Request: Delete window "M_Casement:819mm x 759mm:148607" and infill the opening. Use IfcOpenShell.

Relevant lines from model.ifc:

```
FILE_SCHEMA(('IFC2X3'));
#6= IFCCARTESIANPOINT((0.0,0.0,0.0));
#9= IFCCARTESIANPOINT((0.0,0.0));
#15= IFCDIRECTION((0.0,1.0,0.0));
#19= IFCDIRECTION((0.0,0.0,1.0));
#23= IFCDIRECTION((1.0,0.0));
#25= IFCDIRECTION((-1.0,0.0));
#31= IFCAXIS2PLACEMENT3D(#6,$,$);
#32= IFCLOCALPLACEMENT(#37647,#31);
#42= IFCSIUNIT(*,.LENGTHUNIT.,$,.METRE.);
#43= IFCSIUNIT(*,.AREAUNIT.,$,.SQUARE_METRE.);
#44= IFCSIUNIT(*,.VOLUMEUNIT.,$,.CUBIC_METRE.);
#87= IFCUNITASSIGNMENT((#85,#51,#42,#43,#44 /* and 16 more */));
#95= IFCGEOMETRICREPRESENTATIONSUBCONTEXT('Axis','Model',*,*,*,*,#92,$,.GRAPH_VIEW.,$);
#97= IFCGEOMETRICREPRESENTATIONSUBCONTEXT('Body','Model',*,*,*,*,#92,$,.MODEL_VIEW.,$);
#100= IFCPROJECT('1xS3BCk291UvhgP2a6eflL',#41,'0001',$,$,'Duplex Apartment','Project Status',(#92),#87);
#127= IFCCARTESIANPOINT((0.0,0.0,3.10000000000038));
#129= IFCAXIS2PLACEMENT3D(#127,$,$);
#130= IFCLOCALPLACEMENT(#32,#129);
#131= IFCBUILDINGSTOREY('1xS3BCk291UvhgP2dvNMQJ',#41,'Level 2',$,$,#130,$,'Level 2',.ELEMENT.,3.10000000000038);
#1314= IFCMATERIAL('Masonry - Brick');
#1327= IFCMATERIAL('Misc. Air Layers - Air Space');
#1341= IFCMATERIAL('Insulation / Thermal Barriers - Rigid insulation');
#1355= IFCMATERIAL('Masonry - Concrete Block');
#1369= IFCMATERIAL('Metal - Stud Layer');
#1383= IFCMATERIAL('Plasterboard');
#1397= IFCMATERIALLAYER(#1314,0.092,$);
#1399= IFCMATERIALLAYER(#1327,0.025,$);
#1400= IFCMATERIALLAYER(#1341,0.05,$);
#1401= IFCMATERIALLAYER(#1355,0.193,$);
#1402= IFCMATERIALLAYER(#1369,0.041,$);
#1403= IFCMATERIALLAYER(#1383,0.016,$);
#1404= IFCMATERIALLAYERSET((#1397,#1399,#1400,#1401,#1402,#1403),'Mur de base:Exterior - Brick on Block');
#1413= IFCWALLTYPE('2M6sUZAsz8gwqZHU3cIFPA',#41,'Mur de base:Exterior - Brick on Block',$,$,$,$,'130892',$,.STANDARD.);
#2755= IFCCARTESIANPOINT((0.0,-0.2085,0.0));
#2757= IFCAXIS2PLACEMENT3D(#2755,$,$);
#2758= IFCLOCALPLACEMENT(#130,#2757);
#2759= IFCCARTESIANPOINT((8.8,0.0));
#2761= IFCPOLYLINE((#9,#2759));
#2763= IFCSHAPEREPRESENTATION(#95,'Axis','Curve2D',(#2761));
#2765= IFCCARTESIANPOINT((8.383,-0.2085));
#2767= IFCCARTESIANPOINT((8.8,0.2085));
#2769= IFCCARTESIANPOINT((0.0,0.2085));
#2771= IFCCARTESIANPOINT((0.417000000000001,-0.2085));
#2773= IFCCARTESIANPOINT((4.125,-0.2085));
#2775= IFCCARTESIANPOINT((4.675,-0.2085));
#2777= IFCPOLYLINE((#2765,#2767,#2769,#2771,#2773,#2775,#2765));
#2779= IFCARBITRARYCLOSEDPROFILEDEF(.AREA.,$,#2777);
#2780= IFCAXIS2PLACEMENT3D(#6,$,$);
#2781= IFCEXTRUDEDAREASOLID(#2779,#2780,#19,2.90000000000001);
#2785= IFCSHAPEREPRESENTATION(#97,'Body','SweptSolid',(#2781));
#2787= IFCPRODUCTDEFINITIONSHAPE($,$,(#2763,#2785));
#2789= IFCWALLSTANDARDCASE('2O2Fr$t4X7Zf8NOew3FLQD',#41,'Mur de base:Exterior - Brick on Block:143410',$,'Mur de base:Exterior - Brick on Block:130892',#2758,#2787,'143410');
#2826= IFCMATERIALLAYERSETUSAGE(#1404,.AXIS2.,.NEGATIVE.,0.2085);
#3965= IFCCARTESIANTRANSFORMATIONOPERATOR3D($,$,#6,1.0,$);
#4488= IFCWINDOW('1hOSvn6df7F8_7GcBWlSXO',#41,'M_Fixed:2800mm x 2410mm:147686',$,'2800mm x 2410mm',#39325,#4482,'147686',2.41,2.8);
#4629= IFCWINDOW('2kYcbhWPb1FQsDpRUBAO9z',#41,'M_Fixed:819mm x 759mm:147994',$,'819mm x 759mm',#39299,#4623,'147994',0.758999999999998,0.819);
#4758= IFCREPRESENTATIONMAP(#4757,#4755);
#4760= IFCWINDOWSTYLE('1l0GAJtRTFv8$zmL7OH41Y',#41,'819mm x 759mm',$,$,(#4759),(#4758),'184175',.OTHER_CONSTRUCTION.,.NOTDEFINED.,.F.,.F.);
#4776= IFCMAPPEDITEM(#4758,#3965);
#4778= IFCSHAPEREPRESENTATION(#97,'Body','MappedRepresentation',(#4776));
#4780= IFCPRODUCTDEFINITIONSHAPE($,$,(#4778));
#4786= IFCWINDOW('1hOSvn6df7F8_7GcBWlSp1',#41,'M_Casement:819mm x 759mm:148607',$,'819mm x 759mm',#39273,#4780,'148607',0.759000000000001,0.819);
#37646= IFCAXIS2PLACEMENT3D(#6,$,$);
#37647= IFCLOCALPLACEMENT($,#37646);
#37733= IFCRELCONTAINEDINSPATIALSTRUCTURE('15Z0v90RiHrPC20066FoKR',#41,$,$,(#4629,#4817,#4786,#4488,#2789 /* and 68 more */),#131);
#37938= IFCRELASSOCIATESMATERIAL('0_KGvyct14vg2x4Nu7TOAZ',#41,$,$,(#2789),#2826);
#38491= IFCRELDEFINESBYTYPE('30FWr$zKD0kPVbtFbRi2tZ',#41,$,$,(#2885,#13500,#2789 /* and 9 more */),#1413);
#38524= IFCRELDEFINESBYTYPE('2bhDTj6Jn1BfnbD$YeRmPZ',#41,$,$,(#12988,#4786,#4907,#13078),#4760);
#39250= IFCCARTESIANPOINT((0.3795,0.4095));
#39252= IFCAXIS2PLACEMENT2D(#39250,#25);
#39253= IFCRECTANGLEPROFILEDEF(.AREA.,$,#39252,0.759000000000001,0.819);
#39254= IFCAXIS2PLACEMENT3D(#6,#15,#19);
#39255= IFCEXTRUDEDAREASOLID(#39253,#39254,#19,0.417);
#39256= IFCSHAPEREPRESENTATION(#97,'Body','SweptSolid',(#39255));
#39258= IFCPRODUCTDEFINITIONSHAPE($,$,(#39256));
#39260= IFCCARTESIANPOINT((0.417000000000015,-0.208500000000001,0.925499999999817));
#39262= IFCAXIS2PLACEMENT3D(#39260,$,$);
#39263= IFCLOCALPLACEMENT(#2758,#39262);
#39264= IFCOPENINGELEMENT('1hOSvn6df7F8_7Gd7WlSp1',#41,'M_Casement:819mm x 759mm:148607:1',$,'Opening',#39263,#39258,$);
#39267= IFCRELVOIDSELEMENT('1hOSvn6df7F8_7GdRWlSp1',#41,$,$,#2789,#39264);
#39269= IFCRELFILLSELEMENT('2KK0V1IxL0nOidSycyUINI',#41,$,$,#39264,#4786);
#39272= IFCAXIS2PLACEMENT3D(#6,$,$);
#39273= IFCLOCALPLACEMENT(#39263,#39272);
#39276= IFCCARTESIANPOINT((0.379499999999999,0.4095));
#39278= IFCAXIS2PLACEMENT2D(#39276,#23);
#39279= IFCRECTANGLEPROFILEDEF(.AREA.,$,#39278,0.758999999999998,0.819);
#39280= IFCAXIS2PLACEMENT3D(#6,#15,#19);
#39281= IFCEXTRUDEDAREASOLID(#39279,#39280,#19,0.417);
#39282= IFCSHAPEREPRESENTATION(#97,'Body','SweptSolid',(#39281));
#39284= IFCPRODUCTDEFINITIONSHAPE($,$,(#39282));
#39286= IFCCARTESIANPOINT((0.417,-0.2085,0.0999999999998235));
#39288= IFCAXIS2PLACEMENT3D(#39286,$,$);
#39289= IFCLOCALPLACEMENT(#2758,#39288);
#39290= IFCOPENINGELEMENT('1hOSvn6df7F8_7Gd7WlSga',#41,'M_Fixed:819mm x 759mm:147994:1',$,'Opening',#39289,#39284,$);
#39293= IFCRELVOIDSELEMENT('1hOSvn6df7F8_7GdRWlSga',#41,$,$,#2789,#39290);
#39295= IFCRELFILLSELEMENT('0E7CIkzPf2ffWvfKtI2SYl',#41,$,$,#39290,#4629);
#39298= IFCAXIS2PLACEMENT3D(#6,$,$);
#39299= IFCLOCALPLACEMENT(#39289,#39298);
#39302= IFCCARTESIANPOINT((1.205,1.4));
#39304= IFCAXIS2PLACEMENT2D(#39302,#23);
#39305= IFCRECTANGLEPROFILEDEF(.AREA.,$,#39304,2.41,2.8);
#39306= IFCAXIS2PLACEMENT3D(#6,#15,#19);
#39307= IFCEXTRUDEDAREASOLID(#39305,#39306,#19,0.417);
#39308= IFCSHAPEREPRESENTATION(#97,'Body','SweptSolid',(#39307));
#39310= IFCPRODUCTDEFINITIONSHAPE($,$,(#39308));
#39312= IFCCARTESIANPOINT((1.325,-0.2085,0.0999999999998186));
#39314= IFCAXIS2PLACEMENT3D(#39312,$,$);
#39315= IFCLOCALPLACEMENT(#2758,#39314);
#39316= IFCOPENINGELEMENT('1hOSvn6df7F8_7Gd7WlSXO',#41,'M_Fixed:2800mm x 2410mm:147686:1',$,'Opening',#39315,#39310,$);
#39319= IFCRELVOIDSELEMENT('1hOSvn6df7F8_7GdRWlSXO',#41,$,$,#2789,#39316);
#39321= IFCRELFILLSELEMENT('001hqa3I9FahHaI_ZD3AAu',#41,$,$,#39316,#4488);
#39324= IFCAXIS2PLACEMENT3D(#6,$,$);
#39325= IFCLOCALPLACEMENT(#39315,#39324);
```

```python
import ifcopenshell
import ifcopenshell.api.feature
import ifcopenshell.api.root
import ifcopenshell.geom
import ifcopenshell.util.shape

model = ifcopenshell.open("model.ifc")
settings = ifcopenshell.geom.settings()


def volume(element):
    """Net volume in cubic metres, openings subtracted."""
    shape = ifcopenshell.geom.create_shape(settings, element)
    return ifcopenshell.util.shape.get_volume(shape.geometry)


window = model.by_guid("1hOSvn6df7F8_7GcBWlSp1")
opening = window.FillsVoids[0].RelatingOpeningElement
wall = opening.VoidsElements[0].RelatingBuildingElement
before = volume(wall)

ifcopenshell.api.root.remove_product(model, product=window)
ifcopenshell.api.feature.remove_feature(model, feature=opening)

after = volume(wall)

print(f"wall volume {before:.3f} -> {after:.3f} m3")

model.write("model_updated.ifc")
```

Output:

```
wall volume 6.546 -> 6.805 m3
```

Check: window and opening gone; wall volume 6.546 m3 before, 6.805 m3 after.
